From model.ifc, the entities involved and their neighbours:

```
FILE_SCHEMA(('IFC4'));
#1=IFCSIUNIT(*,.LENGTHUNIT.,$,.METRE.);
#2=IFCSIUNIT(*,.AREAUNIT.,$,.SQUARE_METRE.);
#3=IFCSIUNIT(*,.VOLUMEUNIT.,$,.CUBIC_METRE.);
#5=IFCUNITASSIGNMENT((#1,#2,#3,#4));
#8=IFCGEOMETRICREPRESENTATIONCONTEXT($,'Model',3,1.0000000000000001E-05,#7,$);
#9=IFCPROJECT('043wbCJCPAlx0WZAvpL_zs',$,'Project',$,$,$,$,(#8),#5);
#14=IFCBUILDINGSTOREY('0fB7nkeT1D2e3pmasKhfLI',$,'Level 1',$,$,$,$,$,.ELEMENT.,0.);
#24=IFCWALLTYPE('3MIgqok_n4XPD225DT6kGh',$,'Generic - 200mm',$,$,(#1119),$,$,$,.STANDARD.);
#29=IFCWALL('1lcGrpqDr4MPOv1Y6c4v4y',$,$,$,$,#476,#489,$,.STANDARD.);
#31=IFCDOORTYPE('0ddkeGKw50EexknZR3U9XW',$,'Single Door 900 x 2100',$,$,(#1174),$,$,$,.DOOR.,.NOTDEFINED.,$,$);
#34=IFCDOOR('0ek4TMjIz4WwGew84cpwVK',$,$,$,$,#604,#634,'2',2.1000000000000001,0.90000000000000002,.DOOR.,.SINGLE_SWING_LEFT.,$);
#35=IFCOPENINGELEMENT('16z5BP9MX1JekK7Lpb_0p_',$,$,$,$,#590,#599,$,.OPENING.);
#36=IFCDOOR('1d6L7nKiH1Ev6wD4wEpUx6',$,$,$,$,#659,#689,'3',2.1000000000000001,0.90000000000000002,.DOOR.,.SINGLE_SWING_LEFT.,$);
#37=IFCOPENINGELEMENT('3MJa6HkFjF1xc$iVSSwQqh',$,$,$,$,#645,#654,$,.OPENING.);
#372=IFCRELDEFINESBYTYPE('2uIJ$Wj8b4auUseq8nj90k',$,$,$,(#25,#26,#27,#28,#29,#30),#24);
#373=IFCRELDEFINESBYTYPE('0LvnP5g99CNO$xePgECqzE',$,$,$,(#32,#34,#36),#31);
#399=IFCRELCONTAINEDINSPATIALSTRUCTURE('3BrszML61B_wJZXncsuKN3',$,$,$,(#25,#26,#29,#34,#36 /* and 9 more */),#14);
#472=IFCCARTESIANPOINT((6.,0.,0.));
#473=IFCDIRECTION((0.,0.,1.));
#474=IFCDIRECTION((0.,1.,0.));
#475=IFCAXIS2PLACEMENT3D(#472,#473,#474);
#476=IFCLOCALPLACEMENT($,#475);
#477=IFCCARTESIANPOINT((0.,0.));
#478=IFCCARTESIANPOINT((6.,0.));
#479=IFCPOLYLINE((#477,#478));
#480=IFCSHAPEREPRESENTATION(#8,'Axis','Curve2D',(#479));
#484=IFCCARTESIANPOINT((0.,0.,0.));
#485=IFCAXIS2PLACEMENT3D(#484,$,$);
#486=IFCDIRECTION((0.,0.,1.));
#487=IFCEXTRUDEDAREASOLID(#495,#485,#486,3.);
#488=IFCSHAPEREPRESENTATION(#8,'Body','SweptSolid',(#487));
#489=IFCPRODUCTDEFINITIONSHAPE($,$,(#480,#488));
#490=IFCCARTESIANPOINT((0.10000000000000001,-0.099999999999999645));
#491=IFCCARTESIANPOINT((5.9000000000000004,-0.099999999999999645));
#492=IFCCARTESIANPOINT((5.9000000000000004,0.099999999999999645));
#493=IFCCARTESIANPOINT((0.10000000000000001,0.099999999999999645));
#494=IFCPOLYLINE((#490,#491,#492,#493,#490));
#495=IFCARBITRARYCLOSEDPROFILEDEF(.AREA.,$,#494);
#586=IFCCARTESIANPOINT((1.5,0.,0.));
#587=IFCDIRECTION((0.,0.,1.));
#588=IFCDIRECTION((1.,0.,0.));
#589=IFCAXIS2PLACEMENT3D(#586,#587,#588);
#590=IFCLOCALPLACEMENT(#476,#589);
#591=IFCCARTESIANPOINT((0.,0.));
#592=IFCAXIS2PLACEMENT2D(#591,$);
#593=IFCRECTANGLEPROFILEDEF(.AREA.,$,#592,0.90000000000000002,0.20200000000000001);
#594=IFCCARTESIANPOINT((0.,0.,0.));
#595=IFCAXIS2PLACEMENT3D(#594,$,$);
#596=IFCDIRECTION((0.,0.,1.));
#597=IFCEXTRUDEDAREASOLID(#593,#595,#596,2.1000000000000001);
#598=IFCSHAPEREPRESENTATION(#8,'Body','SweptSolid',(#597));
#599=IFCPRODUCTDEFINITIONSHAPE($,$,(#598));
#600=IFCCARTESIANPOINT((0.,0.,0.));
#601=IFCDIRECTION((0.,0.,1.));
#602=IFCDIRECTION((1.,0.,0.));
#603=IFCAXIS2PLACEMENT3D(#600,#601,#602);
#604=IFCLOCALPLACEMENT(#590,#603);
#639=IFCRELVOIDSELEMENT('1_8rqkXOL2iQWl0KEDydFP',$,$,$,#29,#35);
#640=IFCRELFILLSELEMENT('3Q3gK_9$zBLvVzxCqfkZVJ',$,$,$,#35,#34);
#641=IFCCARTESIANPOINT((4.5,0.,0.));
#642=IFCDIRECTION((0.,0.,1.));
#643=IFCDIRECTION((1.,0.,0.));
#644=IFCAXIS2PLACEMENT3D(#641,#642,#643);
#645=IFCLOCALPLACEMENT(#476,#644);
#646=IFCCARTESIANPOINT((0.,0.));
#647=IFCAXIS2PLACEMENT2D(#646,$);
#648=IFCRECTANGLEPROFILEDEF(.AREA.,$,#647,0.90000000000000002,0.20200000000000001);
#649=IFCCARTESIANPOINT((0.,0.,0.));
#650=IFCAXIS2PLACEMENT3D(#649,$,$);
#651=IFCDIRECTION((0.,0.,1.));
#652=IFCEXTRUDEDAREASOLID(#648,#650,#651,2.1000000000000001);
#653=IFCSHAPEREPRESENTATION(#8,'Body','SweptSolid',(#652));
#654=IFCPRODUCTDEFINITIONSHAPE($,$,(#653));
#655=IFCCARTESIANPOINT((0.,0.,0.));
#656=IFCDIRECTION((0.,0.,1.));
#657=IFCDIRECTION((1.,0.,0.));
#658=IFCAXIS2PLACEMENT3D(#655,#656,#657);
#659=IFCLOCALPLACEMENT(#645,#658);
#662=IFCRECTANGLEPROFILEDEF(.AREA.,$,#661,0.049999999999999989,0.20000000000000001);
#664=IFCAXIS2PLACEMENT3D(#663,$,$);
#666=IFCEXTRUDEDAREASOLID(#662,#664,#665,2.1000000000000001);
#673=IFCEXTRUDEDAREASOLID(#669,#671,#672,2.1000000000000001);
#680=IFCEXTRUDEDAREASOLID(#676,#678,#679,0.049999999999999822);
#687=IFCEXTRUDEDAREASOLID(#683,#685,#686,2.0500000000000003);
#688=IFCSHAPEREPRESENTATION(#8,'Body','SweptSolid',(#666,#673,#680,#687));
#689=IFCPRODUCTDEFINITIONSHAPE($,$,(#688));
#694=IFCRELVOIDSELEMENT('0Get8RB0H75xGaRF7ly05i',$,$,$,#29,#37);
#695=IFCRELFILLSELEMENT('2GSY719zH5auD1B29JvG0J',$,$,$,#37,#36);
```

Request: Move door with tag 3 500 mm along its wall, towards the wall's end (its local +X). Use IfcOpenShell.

```python
import ifcopenshell
import ifcopenshell.api.geometry
import ifcopenshell.util.placement

model = ifcopenshell.open("model.ifc")

door = model.by_guid("1d6L7nKiH1Ev6wD4wEpUx6")
opening = door.FillsVoids[0].RelatingOpeningElement
wall = opening.VoidsElements[0].RelatingBuildingElement

wall_matrix = ifcopenshell.util.placement.get_local_placement(wall.ObjectPlacement)
shift = wall_matrix[:3, 0] * 0.5
before = ifcopenshell.util.placement.get_local_placement(door.ObjectPlacement)[:3, 3].copy()

# The door is placed relative to its opening, so it follows when the opening moves.
matrix = ifcopenshell.util.placement.get_local_placement(opening.ObjectPlacement)
matrix[:3, 3] += shift
ifcopenshell.api.geometry.edit_object_placement(
    model, product=opening, matrix=matrix, is_si=False, should_transform_children=True
)

after = ifcopenshell.util.placement.get_local_placement(door.ObjectPlacement)[:3, 3]
print("door moved by", (after - before).round(3) + 0.0)

model.write("model-out.ifc")
```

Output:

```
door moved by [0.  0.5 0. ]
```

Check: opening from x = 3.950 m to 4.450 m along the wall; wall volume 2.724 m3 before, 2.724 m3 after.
